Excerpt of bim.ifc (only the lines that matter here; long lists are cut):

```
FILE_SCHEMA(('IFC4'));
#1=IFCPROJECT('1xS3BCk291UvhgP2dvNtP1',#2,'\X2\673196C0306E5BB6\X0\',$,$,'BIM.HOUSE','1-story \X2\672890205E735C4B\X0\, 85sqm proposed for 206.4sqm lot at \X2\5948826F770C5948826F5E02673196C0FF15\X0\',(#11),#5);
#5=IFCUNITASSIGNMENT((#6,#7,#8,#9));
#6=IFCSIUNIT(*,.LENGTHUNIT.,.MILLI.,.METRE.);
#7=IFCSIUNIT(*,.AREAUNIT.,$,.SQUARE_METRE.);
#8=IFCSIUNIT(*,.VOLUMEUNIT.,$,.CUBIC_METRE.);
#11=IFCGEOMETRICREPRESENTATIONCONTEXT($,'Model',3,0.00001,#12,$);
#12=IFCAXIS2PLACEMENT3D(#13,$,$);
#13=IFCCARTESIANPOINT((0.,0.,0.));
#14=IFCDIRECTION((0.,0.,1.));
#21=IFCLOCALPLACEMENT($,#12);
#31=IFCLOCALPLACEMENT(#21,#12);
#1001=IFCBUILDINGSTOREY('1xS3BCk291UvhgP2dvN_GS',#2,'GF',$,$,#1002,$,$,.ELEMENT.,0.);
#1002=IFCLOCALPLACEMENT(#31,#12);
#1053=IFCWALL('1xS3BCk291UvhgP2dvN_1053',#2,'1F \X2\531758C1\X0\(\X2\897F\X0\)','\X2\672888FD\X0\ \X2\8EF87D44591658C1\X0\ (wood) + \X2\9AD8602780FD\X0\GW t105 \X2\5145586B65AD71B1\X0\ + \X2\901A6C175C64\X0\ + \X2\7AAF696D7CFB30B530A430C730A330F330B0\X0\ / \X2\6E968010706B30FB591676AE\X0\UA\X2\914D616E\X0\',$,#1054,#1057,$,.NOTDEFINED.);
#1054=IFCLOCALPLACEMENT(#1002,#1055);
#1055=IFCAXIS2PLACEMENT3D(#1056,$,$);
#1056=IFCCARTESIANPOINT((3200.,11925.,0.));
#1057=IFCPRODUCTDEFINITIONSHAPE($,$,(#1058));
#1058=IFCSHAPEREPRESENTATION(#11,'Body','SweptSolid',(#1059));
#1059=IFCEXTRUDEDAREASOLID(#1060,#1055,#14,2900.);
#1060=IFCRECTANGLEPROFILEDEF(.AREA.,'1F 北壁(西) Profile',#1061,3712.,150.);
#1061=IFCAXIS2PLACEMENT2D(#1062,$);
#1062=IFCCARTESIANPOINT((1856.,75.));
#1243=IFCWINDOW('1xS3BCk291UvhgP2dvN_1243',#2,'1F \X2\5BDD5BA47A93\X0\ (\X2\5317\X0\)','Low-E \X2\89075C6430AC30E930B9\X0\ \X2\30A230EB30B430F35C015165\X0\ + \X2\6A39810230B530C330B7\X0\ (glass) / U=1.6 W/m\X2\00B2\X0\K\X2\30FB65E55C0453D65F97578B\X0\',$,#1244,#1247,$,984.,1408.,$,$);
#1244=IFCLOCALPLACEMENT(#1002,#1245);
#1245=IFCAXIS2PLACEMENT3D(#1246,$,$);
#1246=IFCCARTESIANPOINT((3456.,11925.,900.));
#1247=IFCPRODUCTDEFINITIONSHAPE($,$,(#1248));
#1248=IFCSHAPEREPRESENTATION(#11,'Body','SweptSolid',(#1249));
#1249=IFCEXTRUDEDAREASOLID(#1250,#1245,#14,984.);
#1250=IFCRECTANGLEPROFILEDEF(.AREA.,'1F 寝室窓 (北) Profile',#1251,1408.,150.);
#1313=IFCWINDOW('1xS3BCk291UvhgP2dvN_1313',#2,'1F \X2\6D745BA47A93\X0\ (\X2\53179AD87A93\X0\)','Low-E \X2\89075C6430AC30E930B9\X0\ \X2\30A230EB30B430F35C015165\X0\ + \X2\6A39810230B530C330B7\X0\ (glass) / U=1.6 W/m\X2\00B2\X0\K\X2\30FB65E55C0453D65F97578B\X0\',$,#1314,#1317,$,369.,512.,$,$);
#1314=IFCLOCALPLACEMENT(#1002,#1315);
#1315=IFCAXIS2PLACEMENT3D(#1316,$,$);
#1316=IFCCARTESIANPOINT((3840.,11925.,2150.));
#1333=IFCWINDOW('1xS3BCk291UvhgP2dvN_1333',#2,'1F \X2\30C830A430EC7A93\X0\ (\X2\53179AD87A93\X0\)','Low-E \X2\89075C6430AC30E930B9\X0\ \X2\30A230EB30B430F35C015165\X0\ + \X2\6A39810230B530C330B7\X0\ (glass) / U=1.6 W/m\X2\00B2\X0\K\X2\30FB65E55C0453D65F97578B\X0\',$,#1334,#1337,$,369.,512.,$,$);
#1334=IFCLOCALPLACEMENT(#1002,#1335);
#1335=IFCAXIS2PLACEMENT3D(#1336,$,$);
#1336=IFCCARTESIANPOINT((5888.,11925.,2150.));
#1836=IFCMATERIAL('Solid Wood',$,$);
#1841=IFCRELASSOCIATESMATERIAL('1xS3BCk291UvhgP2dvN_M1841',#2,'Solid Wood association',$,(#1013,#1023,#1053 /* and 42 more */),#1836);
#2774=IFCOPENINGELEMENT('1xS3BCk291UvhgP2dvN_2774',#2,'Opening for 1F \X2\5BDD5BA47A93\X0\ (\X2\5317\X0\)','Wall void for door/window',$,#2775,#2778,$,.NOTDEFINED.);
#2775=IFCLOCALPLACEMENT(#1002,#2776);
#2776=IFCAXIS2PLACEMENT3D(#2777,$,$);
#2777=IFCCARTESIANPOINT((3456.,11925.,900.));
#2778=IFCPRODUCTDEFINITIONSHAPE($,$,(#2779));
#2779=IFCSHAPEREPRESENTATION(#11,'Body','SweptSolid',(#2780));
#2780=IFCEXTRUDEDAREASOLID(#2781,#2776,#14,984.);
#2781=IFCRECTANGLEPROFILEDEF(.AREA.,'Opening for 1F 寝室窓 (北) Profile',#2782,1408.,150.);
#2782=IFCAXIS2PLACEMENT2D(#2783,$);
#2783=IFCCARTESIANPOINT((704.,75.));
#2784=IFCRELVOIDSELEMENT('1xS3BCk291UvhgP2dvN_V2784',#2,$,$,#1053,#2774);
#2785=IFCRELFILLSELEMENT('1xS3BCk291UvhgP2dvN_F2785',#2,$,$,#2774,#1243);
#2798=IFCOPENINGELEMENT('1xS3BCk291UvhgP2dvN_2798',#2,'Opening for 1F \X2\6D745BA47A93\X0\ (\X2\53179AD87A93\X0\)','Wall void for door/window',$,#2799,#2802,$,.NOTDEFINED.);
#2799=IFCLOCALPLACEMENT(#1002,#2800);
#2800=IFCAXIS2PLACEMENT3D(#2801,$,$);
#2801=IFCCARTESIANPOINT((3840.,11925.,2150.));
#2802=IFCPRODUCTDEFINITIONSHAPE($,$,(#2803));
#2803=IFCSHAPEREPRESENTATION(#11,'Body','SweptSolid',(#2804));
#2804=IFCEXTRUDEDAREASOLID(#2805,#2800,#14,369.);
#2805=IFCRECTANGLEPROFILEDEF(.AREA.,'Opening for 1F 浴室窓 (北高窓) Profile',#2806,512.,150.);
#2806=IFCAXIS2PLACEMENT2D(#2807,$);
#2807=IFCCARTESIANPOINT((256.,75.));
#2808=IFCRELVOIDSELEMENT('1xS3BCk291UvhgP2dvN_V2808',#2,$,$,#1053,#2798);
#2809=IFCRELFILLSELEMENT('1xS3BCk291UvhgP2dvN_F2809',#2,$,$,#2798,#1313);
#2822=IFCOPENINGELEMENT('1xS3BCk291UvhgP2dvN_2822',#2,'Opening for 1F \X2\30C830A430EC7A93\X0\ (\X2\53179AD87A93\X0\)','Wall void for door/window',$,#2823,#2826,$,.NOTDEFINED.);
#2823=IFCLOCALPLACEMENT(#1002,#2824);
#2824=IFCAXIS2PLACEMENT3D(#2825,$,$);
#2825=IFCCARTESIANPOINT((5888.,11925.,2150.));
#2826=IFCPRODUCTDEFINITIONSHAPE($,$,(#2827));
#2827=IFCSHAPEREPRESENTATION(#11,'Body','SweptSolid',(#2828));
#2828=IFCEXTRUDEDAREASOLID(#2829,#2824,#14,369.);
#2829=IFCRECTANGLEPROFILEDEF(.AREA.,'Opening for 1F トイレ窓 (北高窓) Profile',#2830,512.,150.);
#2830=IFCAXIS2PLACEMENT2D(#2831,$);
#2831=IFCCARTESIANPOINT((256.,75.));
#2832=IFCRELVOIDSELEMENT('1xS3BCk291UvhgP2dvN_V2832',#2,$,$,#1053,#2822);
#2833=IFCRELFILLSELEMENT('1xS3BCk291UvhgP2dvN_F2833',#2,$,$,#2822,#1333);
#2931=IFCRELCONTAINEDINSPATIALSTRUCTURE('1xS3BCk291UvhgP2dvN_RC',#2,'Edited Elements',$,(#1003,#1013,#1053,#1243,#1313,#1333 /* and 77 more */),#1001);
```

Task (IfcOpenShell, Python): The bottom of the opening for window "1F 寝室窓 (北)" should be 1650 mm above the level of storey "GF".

```python
import numpy as np
import ifcopenshell
import ifcopenshell.api.geometry
import ifcopenshell.geom
import ifcopenshell.util.element
import ifcopenshell.util.placement
import ifcopenshell.util.shape
import ifcopenshell.util.unit

model = ifcopenshell.open("bim.ifc")
unit_scale = ifcopenshell.util.unit.calculate_unit_scale(model)

window = model.by_id(1243)
opening = window.FillsVoids[0].RelatingOpeningElement
storey = ifcopenshell.util.element.get_container(window, ifc_class="IfcBuildingStorey")
level = ifcopenshell.util.placement.get_local_placement(storey.ObjectPlacement)[2, 3]

# The opening's origin need not be at the sill, so measure its lowest point.
shape = ifcopenshell.geom.create_shape(ifcopenshell.geom.settings(), opening)
bottom = ifcopenshell.util.shape.get_shape_bottom_elevation(shape, shape.geometry) / unit_scale
dz = level + 1.65 / unit_scale - bottom

shift = np.array([0.0, 0.0, dz])
# The window is not placed relative to its opening, so move both.
for product in (opening, window):
    matrix = ifcopenshell.util.placement.get_local_placement(product.ObjectPlacement)
    matrix[:3, 3] += shift
    ifcopenshell.api.geometry.edit_object_placement(model, product=product, matrix=matrix, is_si=False)

print(f"moved by {dz * unit_scale:+.3f} m")

model.write("bim_updated.ifc")
```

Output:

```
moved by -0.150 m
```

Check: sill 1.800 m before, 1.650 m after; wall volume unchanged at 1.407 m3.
